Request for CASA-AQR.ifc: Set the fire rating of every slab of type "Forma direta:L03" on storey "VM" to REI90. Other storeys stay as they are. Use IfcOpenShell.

First a look at what the model holds.

```python
import ifcopenshell
import ifcopenshell.util.element

model = ifcopenshell.open("CASA-AQR.ifc")
print(model.schema)
storey = next(s for s in model.by_type("IfcBuildingStorey") if s.Name == "VM")
slabs = [e for e in ifcopenshell.util.element.get_decomposition(storey) if e.is_a("IfcSlab")]
seen = {}
for e in slabs:
    element_type = ifcopenshell.util.element.get_type(e)
    key = (element_type.Name if element_type != e and element_type else None, ifcopenshell.util.element.get_pset(e, "Pset_SlabCommon", "FireRating"))
    seen[key] = seen.get(key, 0) + 1
for (name, value), count in sorted(seen.items(), key=str):
    print(count, "x", name, "|", value)
```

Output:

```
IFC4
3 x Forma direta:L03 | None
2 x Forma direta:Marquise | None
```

```python
import ifcopenshell
import ifcopenshell.api.pset
import ifcopenshell.util.element

model = ifcopenshell.open("CASA-AQR.ifc")

storey = next(s for s in model.by_type("IfcBuildingStorey") if s.Name == "VM")
slabs = [e for e in ifcopenshell.util.element.get_decomposition(storey) if e.is_a("IfcSlab")]

count = 0
for e in slabs:
    element_type = ifcopenshell.util.element.get_type(e)
    if element_type in (None, e) or element_type.Name != "Forma direta:L03":
        continue
    # add_pset returns the element's existing set when there is one.
    pset = ifcopenshell.api.pset.add_pset(model, product=e, name="Pset_SlabCommon")
    ifcopenshell.api.pset.edit_pset(model, pset=pset, properties={"FireRating": "REI90"})
    count += 1

print(count, "slabs updated")

model.write("CASA-AQR_updated.ifc")
```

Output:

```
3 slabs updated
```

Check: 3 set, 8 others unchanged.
